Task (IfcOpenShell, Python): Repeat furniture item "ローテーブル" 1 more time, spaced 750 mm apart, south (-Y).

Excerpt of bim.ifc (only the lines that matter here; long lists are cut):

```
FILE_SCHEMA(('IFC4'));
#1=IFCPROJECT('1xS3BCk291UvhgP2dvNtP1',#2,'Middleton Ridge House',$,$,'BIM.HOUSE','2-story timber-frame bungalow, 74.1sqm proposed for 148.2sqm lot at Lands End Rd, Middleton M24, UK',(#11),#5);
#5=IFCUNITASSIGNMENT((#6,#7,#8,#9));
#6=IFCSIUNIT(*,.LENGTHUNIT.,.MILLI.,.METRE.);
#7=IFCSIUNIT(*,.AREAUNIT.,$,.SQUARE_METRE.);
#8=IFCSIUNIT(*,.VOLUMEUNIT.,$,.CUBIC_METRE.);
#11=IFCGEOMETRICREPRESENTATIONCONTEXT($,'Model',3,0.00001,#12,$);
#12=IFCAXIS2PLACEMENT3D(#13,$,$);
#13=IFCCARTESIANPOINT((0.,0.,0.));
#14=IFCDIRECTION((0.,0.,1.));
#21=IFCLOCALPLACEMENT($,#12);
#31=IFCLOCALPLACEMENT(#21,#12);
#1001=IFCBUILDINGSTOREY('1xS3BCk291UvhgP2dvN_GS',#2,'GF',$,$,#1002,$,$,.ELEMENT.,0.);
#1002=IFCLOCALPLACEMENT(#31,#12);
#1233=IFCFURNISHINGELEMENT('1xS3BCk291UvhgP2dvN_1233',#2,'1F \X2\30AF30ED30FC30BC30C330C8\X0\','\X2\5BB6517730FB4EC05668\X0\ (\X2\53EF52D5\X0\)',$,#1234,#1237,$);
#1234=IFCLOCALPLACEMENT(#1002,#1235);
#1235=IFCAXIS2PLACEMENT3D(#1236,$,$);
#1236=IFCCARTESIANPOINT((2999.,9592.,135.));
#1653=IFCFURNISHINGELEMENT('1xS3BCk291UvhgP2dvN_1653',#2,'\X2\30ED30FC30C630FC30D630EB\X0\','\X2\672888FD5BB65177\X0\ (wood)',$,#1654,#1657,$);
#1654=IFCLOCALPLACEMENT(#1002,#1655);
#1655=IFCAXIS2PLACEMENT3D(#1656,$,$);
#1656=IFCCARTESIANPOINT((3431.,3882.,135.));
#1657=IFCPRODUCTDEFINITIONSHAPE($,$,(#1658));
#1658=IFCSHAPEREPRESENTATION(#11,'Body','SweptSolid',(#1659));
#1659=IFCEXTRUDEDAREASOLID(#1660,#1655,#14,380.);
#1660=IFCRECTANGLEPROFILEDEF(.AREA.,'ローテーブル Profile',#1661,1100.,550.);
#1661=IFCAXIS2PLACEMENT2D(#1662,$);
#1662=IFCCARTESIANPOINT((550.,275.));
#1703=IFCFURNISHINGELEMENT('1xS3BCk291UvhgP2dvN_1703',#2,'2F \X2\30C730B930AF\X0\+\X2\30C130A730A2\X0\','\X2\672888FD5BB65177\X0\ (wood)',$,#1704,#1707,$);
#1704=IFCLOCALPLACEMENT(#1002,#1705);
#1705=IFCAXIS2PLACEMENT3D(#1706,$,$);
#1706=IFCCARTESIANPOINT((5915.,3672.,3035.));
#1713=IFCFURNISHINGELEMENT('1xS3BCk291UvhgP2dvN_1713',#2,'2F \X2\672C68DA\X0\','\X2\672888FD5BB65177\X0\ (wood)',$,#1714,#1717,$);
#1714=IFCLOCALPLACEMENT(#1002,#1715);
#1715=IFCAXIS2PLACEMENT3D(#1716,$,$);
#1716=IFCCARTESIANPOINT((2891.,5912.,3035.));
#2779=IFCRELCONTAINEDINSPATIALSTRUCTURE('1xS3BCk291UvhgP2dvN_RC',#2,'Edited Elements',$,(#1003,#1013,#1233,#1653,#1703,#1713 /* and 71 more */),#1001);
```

```python
import numpy as np
import ifcopenshell
import ifcopenshell.api.geometry
import ifcopenshell.api.root
import ifcopenshell.util.element
import ifcopenshell.util.placement
import ifcopenshell.util.unit

model = ifcopenshell.open("bim.ifc")
unit_scale = ifcopenshell.util.unit.calculate_unit_scale(model)


def reuse_history(source, copy):
    """copy_class also copies each property set's owner history, people and application; keep the originals."""
    for rel in copy.IsDefinedBy:
        if rel.is_a("IfcRelDefinesByProperties") and (history := rel.RelatingPropertyDefinition.OwnerHistory):
            rel.RelatingPropertyDefinition.OwnerHistory = source.OwnerHistory
            ifcopenshell.util.element.remove_deep2(model, history)


source = model.by_guid("1xS3BCk291UvhgP2dvN_1653")
base = ifcopenshell.util.placement.get_local_placement(source.ObjectPlacement)
step = np.array([0.0, -1.0, 0.0]) * 0.75 / unit_scale

for i in range(1, 2):
    copy = ifcopenshell.api.root.copy_class(model, product=source)
    copy.Representation = ifcopenshell.util.element.copy_deep(
        model, source.Representation, exclude=["IfcGeometricRepresentationContext", "IfcRepresentationMap"]
    )
    reuse_history(source, copy)
    matrix = base.copy()
    matrix[:3, 3] += i * step
    print("added at", matrix[:3, 3].round(3) + 0.0)
    ifcopenshell.api.geometry.edit_object_placement(model, product=copy, matrix=matrix, is_si=False)

model.write("bim_edited.ifc")
```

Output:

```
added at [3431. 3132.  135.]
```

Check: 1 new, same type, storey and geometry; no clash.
